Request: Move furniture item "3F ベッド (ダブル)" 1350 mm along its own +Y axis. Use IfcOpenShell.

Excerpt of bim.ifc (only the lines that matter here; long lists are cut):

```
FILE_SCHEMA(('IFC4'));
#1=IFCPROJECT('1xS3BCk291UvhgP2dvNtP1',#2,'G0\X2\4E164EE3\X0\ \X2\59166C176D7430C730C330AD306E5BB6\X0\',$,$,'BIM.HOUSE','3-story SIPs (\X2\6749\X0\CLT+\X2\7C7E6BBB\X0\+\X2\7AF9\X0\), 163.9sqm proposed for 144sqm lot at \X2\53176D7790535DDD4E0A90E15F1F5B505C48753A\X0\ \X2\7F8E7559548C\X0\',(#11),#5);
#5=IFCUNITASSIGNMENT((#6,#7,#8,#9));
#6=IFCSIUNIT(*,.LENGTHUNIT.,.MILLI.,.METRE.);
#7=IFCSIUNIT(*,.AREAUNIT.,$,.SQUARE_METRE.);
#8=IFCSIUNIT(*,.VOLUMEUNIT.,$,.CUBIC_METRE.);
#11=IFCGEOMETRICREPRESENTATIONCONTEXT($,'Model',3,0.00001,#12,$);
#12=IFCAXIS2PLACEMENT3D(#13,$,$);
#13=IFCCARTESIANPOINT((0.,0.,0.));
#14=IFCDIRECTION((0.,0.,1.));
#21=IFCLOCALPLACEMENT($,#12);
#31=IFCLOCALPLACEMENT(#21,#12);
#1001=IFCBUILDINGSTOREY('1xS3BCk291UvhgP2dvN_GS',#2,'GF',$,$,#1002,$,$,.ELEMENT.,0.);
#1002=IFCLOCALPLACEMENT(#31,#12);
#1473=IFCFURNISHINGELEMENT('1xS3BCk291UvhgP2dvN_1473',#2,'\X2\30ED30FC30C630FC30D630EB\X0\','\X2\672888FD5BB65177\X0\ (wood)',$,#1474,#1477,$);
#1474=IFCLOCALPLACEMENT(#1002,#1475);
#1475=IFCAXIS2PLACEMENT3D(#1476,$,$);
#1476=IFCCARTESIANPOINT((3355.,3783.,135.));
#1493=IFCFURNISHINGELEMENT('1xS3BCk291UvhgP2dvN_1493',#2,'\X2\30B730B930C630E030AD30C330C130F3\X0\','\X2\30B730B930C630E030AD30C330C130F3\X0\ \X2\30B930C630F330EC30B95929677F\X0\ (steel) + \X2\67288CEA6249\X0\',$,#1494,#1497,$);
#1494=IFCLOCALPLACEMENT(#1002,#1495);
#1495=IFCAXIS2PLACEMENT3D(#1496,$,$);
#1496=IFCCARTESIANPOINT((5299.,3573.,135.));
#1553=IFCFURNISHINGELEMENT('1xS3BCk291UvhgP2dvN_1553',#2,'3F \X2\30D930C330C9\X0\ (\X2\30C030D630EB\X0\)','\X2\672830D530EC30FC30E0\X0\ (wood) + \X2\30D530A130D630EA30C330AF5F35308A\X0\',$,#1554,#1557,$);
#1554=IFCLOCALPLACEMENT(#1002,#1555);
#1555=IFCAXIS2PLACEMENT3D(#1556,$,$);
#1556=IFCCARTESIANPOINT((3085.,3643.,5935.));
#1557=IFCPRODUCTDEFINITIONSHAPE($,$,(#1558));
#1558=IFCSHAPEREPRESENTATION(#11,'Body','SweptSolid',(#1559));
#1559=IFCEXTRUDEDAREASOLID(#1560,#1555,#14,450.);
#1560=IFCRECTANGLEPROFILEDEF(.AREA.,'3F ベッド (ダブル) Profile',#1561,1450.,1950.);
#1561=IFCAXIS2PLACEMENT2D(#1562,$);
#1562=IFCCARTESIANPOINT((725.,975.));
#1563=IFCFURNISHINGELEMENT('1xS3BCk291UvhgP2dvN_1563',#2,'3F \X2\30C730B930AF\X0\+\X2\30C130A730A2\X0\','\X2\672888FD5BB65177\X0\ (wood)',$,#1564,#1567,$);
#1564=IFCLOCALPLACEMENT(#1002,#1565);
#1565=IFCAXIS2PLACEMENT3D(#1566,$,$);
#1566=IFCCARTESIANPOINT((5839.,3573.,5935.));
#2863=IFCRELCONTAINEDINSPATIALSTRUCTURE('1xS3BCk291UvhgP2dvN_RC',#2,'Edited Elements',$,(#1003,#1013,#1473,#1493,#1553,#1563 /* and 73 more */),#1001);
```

```python
import ifcopenshell
import ifcopenshell.api.geometry
import ifcopenshell.util.placement
import ifcopenshell.util.unit

model = ifcopenshell.open("bim.ifc")
unit_scale = ifcopenshell.util.unit.calculate_unit_scale(model)

item = model.by_id(1553)
matrix = ifcopenshell.util.placement.get_local_placement(item.ObjectPlacement)
matrix[:3, 3] += matrix[:3, 1] * 1.35 / unit_scale
ifcopenshell.api.geometry.edit_object_placement(model, product=item, matrix=matrix, is_si=False)

print(ifcopenshell.util.placement.get_local_placement(item.ObjectPlacement).round(3) + 0.0)

model.write("bim-out.ifc")
```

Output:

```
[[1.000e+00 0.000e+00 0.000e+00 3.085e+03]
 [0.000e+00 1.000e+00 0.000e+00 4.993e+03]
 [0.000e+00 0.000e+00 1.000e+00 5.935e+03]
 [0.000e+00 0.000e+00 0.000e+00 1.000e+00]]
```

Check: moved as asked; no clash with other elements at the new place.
